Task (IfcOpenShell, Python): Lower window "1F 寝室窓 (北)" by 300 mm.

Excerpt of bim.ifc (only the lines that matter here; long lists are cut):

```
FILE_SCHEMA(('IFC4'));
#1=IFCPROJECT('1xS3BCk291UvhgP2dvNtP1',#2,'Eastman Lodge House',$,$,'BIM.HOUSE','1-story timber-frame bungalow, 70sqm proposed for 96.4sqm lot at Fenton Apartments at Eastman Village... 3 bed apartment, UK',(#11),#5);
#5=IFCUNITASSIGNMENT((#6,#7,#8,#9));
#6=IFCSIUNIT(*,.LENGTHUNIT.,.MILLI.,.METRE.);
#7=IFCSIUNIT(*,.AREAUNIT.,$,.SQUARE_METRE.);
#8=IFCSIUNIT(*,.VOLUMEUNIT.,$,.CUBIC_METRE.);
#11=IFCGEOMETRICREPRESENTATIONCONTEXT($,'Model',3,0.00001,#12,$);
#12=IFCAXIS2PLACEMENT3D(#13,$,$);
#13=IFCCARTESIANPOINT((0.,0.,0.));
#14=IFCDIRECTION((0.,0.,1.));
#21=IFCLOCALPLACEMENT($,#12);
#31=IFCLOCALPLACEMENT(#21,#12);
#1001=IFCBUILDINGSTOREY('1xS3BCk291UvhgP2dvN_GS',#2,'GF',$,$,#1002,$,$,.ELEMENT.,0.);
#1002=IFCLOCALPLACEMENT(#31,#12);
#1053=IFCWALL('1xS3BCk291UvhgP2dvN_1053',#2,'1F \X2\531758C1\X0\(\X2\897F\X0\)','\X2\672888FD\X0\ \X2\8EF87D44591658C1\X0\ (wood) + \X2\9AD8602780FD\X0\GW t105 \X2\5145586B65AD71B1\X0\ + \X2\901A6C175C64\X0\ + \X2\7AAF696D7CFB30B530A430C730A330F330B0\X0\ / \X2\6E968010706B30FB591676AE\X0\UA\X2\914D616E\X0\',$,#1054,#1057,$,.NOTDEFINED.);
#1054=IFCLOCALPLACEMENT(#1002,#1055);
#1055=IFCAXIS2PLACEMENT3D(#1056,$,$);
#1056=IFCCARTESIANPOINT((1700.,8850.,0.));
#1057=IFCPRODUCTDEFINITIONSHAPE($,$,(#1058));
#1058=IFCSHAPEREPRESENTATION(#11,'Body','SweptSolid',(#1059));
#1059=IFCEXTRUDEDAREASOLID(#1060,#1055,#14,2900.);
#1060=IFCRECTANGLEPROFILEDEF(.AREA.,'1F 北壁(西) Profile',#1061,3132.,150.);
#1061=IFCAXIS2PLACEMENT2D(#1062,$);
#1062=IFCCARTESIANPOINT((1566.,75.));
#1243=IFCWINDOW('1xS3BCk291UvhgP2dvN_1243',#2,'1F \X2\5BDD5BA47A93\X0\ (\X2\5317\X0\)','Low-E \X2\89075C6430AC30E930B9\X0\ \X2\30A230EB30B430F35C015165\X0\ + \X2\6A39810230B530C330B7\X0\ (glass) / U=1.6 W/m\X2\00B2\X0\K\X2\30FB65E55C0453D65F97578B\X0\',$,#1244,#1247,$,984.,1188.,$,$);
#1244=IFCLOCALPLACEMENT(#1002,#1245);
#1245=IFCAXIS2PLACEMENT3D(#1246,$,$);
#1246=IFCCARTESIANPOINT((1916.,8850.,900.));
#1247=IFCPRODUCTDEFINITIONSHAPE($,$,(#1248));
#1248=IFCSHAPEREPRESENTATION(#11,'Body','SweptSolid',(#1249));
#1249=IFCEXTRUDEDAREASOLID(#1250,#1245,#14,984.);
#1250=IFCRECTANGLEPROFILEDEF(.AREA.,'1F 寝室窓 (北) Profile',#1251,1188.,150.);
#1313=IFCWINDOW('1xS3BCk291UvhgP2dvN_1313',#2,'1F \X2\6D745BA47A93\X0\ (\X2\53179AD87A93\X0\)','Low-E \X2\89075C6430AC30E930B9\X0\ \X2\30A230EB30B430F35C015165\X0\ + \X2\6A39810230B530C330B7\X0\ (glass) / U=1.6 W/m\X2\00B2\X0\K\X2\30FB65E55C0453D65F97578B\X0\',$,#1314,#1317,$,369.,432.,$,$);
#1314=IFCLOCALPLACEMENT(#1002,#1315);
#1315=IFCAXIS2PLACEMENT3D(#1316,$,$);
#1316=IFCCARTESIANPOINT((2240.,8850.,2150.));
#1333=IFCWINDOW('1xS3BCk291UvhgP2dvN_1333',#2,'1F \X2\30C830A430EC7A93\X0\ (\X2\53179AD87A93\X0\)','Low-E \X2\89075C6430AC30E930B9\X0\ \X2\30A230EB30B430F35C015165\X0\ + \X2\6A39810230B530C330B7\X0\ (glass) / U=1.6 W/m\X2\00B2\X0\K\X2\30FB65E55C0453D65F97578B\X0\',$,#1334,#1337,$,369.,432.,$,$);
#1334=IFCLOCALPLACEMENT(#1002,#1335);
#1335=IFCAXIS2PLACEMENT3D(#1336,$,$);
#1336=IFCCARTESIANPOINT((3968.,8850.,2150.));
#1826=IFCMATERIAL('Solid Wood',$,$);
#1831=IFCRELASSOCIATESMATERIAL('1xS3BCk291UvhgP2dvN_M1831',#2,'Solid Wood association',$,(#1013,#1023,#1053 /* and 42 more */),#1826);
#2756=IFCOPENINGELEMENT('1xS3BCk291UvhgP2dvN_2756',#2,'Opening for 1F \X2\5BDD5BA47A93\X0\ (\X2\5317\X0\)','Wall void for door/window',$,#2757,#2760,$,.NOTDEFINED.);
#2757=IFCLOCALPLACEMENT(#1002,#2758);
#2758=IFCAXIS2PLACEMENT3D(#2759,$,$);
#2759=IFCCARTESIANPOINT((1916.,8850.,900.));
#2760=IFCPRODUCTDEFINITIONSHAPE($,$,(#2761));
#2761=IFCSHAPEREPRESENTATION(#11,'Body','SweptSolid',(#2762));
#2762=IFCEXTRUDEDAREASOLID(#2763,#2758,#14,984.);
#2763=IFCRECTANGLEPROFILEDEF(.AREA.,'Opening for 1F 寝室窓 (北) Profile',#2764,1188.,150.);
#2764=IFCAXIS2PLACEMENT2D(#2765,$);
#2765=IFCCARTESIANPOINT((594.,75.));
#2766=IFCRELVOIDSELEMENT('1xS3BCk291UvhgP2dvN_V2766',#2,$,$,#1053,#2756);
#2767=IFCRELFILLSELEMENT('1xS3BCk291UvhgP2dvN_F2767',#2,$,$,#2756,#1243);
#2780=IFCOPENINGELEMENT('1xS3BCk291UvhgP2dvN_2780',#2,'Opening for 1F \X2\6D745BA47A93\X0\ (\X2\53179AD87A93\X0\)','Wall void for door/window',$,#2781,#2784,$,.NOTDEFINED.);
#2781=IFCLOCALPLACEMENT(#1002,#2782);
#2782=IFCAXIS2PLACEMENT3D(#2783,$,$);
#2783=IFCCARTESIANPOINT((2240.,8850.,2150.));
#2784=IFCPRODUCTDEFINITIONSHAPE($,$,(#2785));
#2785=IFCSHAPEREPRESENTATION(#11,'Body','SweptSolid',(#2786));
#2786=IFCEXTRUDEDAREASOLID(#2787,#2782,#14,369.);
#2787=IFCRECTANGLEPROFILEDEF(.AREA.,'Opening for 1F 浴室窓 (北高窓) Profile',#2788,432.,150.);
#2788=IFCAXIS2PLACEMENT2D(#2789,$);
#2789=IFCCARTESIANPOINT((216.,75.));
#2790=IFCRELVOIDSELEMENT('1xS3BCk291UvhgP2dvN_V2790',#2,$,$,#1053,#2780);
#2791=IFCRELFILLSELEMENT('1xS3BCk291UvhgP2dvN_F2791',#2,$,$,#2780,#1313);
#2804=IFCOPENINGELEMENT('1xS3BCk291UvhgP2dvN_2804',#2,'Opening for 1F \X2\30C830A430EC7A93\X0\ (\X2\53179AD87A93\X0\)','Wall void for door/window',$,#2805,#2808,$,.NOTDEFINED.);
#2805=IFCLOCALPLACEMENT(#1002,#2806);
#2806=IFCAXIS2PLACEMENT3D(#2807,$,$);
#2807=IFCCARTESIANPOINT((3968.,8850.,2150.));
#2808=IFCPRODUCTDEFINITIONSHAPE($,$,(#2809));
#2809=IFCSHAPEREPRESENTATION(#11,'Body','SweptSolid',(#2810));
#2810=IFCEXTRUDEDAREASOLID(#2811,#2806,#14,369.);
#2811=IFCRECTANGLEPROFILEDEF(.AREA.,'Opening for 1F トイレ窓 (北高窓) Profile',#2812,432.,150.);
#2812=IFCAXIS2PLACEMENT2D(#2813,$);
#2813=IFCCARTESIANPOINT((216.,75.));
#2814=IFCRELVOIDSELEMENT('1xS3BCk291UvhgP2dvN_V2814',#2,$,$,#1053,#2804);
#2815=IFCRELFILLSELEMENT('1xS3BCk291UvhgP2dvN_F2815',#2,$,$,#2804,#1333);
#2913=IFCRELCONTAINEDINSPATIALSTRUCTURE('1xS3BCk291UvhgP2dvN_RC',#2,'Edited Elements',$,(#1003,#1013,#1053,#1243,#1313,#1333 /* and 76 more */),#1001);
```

```python
import numpy as np
import ifcopenshell
import ifcopenshell.api.geometry
import ifcopenshell.util.placement
import ifcopenshell.util.unit

model = ifcopenshell.open("bim.ifc")
unit_scale = ifcopenshell.util.unit.calculate_unit_scale(model)

window = model.by_guid("1xS3BCk291UvhgP2dvN_1243")
opening = window.FillsVoids[0].RelatingOpeningElement
dz = -0.3 / unit_scale

shift = np.array([0.0, 0.0, dz])
# The window is not placed relative to its opening, so move both.
for product in (opening, window):
    matrix = ifcopenshell.util.placement.get_local_placement(product.ObjectPlacement)
    matrix[:3, 3] += shift
    ifcopenshell.api.geometry.edit_object_placement(model, product=product, matrix=matrix, is_si=False)

print(f"moved by {dz * unit_scale:+.3f} m")

model.write("bim_updated.ifc")
```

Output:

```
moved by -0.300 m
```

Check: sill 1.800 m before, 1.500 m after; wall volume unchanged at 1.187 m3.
